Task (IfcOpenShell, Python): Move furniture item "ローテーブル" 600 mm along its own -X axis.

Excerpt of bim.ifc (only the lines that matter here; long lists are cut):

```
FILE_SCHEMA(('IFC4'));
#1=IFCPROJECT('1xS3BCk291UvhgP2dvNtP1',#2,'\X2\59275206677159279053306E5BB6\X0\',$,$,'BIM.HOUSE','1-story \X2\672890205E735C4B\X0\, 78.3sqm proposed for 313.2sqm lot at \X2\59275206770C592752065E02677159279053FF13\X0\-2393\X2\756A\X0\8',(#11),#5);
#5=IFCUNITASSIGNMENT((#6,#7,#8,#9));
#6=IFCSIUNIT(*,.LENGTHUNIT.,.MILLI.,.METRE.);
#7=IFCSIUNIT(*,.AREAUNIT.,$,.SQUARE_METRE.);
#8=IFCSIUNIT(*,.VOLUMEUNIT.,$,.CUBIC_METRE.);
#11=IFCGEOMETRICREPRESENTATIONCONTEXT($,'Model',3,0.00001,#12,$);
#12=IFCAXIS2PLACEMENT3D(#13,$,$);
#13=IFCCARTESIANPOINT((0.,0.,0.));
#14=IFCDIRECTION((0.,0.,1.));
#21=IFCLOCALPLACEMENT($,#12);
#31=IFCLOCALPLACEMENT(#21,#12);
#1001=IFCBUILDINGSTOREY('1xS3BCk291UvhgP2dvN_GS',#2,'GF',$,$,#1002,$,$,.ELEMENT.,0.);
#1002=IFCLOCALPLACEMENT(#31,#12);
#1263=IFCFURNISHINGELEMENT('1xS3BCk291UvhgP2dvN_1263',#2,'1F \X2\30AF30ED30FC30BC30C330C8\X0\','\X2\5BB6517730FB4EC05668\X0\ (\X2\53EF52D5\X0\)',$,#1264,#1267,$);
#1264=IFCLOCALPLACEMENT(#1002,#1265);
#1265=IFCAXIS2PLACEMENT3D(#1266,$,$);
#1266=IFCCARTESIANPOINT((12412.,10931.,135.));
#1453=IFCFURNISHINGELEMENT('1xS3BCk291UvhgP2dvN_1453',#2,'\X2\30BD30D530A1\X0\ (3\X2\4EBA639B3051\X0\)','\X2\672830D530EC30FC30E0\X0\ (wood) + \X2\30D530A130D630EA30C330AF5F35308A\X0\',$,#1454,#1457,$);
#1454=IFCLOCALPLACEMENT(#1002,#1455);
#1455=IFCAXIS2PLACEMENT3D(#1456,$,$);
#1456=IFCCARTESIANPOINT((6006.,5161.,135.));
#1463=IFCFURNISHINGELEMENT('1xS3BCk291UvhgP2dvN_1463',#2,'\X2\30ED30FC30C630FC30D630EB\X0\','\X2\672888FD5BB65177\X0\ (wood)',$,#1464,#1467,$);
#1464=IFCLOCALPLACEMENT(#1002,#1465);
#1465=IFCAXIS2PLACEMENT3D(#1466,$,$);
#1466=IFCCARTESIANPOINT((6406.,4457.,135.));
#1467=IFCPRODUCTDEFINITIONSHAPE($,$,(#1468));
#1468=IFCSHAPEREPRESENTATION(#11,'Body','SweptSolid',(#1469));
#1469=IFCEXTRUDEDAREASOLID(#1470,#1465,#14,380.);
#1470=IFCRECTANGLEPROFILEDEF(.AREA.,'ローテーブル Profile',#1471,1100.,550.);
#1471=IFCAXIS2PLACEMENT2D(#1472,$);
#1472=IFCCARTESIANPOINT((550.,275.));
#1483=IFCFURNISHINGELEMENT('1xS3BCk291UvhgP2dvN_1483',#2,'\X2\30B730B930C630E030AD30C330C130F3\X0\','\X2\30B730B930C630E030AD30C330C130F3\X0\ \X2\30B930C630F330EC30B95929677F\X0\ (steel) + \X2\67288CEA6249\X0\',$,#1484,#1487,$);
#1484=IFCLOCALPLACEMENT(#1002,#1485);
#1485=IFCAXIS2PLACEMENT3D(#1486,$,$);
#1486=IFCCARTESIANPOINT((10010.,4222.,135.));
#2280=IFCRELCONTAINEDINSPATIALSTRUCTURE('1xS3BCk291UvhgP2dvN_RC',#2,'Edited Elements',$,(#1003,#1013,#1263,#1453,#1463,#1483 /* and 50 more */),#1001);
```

```python
import ifcopenshell
import ifcopenshell.api.geometry
import ifcopenshell.util.placement
import ifcopenshell.util.unit

model = ifcopenshell.open("bim.ifc")
unit_scale = ifcopenshell.util.unit.calculate_unit_scale(model)

item = model.by_guid("1xS3BCk291UvhgP2dvN_1463")
matrix = ifcopenshell.util.placement.get_local_placement(item.ObjectPlacement)
matrix[:3, 3] -= matrix[:3, 0] * 0.6 / unit_scale
ifcopenshell.api.geometry.edit_object_placement(model, product=item, matrix=matrix, is_si=False)

print(ifcopenshell.util.placement.get_local_placement(item.ObjectPlacement).round(3) + 0.0)

model.write("bim-out.ifc")
```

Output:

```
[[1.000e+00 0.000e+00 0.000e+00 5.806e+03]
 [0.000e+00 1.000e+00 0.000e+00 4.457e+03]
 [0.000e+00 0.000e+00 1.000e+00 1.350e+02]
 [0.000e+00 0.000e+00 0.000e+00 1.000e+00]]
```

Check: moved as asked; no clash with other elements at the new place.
